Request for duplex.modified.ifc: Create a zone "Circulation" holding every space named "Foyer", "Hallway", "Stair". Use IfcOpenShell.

First a look at what the model holds.

```python
import ifcopenshell

model = ifcopenshell.open("duplex.modified.ifc")
print(model.schema)
seen = {}
for space in model.by_type("IfcSpace"):
    seen[space.LongName] = seen.get(space.LongName, 0) + 1
for name, count in sorted(seen.items(), key=str):
    print(count, "x", name)
print("zones:", [z.Name for z in model.by_type("IfcZone")][:20])
```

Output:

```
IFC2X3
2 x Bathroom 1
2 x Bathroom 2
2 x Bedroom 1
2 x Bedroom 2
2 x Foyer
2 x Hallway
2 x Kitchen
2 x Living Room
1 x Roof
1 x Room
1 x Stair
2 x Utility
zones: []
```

```python
import ifcopenshell
import ifcopenshell.api.group
import ifcopenshell.api.root

model = ifcopenshell.open("duplex.modified.ifc")

names = {"Foyer", "Hallway", "Stair"}
spaces = [s for s in model.by_type("IfcSpace") if s.LongName in names]

zone = ifcopenshell.api.root.create_entity(model, ifc_class="IfcZone", name="Circulation")
ifcopenshell.api.group.assign_group(model, products=spaces, group=zone)
print(len(spaces), "spaces in", zone.Name)

model.write("duplex.modified_updated.ifc")
```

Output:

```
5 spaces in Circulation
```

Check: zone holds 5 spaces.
